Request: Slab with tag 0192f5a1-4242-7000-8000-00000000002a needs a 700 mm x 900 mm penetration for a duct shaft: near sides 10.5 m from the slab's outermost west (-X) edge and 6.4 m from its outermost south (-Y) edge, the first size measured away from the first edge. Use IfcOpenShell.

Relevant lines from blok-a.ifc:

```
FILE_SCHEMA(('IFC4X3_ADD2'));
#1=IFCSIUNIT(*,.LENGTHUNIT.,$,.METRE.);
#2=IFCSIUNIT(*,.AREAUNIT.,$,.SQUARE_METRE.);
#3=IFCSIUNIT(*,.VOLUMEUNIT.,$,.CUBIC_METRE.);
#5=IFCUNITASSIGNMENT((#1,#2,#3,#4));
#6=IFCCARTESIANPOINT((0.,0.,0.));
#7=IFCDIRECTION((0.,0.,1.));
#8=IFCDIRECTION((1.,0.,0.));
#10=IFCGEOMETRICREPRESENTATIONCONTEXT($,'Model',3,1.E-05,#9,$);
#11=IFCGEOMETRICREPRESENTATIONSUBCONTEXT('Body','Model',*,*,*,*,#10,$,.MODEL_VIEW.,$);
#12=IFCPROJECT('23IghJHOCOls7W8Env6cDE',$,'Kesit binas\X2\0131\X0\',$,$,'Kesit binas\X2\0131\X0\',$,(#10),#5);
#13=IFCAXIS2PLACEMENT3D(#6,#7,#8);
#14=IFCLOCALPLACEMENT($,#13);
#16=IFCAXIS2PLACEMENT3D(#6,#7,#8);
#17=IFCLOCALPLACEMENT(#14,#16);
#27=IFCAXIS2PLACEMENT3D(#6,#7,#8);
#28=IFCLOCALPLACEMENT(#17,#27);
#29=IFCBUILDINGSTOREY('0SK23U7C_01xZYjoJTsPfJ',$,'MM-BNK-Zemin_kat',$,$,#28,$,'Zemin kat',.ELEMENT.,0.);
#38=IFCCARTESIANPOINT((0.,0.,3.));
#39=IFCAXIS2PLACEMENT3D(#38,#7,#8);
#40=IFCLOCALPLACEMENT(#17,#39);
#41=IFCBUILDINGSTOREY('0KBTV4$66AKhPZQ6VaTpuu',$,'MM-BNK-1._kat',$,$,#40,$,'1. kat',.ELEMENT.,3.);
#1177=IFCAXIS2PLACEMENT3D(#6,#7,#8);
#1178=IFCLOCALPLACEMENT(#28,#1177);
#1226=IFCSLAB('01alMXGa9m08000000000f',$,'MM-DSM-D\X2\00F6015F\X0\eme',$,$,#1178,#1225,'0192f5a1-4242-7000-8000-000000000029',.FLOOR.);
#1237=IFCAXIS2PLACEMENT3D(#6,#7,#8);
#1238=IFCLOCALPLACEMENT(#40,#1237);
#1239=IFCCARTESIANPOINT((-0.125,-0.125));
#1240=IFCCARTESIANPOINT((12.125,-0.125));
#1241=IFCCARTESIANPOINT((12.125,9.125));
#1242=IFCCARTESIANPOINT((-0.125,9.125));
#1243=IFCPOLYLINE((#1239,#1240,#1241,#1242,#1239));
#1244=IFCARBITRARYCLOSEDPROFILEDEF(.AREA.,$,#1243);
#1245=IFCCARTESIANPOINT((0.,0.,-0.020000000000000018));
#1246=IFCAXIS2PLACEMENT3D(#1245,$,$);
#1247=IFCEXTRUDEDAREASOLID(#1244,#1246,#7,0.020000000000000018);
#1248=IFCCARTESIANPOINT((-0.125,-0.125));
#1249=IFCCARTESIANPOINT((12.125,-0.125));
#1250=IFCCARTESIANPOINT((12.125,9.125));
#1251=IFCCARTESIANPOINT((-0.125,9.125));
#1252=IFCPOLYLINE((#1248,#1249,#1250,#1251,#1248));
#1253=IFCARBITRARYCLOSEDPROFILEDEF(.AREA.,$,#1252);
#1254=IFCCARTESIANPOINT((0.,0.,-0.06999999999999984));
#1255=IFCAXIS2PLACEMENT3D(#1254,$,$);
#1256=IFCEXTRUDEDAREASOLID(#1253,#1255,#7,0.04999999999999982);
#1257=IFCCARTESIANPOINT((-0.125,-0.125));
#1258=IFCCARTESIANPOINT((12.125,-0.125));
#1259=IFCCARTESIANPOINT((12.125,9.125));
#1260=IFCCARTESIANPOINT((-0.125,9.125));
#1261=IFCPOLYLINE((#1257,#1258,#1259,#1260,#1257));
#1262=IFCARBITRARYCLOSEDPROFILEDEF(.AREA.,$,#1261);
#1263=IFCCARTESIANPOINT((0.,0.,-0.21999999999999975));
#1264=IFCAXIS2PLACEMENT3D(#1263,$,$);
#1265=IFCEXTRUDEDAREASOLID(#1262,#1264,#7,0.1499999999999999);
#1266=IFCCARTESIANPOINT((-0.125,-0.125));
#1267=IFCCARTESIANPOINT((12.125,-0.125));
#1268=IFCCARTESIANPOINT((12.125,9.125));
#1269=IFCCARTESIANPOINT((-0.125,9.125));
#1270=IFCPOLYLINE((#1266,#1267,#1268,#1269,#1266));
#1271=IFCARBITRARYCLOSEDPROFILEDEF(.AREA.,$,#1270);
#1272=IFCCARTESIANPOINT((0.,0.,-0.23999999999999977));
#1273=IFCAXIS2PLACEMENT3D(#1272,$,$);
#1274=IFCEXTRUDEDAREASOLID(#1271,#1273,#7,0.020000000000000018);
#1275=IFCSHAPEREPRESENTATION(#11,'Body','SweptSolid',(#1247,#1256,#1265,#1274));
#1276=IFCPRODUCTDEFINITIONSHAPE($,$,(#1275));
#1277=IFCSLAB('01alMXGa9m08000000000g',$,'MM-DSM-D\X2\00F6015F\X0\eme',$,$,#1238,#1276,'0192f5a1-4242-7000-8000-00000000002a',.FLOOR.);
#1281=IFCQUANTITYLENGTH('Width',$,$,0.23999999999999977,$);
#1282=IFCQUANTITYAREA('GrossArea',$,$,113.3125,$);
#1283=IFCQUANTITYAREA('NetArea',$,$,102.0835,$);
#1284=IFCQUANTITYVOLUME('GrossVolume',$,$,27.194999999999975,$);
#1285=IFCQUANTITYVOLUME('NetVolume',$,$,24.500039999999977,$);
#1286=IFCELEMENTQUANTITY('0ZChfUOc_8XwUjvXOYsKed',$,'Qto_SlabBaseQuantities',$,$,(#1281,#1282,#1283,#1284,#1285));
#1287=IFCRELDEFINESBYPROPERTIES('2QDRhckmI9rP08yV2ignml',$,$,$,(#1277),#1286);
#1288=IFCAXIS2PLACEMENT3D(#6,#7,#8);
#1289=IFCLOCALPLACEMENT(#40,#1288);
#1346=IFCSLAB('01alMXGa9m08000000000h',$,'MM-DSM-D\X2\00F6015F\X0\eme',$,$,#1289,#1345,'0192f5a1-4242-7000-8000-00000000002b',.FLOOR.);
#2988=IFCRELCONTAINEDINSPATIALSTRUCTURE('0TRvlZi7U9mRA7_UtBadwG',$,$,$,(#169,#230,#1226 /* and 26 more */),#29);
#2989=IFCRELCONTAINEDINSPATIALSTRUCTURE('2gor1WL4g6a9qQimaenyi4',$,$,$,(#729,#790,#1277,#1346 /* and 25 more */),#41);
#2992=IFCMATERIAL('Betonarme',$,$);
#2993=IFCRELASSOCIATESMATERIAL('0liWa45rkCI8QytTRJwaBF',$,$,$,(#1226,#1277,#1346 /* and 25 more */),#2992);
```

```python
import numpy as np
import ifcopenshell
import ifcopenshell.api.feature
import ifcopenshell.api.geometry
import ifcopenshell.api.pset
import ifcopenshell.api.root
import ifcopenshell.geom
import ifcopenshell.util.element
import ifcopenshell.util.placement
import ifcopenshell.util.representation
import ifcopenshell.util.shape
import ifcopenshell.util.unit

model = ifcopenshell.open("blok-a.ifc")
unit_scale = ifcopenshell.util.unit.calculate_unit_scale(model)
area_scale = ifcopenshell.util.unit.calculate_unit_scale(model, "AREAUNIT")
volume_scale = ifcopenshell.util.unit.calculate_unit_scale(model, "VOLUMEUNIT")
settings = ifcopenshell.geom.settings()


def volume(element):
    """Net volume in cubic metres, openings subtracted."""
    shape = ifcopenshell.geom.create_shape(settings, element)
    return ifcopenshell.util.shape.get_volume(shape.geometry)


slab = model.by_guid("01alMXGa9m08000000000g")
before = volume(slab)

# Extent in the slab's own axes, in metres. The edges named are its -X and -Y sides.
slab_shape = ifcopenshell.geom.create_shape(settings, slab)
vertices = ifcopenshell.util.shape.get_vertices(slab_shape.geometry)
x_min, y_min, bottom = vertices.min(axis=0)
top = vertices[:, 2].max()

opening = ifcopenshell.api.root.create_entity(model, ifc_class="IfcOpeningElement", name="Duct shaft opening", predefined_type="OPENING")
context = ifcopenshell.util.representation.get_context(model, "Model", "Body", "MODEL_VIEW")
width, depth = 0.7, 0.9
outline = [(0.0, 0.0), (width, 0.0), (width, depth), (0.0, depth), (0.0, 0.0)]
# Overshoot both faces by 50 mm so the cut is clean.
shape = ifcopenshell.api.geometry.add_slab_representation(
    model, context=context, depth=top - bottom + 0.1, polyline=outline
)
ifcopenshell.api.geometry.assign_representation(model, product=opening, representation=shape)

matrix = ifcopenshell.util.placement.get_local_placement(slab.ObjectPlacement)
matrix[:, 3] = matrix @ np.append(np.array([x_min + 10.5, y_min + 6.4, bottom - 0.05]) / unit_scale, 1.0)
ifcopenshell.api.geometry.edit_object_placement(model, product=opening, matrix=matrix, is_si=False)
ifcopenshell.api.feature.add_feature(model, feature=opening, element=slab)

after = volume(slab)

# Update the slab's stored quantities.
qto = model.by_id(ifcopenshell.util.element.get_pset(slab, "Qto_SlabBaseQuantities", should_inherit=False)["id"])
ifcopenshell.api.pset.edit_qto(model, qto=qto, properties={
    "NetArea": after / (top - bottom) / area_scale,
    "NetVolume": after / volume_scale,
})

print(f"slab volume {before:.3f} -> {after:.3f} m3")

model.write("blok-a_updated.ifc")
```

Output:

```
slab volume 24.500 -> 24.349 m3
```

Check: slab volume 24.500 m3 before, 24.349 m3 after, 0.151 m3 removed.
